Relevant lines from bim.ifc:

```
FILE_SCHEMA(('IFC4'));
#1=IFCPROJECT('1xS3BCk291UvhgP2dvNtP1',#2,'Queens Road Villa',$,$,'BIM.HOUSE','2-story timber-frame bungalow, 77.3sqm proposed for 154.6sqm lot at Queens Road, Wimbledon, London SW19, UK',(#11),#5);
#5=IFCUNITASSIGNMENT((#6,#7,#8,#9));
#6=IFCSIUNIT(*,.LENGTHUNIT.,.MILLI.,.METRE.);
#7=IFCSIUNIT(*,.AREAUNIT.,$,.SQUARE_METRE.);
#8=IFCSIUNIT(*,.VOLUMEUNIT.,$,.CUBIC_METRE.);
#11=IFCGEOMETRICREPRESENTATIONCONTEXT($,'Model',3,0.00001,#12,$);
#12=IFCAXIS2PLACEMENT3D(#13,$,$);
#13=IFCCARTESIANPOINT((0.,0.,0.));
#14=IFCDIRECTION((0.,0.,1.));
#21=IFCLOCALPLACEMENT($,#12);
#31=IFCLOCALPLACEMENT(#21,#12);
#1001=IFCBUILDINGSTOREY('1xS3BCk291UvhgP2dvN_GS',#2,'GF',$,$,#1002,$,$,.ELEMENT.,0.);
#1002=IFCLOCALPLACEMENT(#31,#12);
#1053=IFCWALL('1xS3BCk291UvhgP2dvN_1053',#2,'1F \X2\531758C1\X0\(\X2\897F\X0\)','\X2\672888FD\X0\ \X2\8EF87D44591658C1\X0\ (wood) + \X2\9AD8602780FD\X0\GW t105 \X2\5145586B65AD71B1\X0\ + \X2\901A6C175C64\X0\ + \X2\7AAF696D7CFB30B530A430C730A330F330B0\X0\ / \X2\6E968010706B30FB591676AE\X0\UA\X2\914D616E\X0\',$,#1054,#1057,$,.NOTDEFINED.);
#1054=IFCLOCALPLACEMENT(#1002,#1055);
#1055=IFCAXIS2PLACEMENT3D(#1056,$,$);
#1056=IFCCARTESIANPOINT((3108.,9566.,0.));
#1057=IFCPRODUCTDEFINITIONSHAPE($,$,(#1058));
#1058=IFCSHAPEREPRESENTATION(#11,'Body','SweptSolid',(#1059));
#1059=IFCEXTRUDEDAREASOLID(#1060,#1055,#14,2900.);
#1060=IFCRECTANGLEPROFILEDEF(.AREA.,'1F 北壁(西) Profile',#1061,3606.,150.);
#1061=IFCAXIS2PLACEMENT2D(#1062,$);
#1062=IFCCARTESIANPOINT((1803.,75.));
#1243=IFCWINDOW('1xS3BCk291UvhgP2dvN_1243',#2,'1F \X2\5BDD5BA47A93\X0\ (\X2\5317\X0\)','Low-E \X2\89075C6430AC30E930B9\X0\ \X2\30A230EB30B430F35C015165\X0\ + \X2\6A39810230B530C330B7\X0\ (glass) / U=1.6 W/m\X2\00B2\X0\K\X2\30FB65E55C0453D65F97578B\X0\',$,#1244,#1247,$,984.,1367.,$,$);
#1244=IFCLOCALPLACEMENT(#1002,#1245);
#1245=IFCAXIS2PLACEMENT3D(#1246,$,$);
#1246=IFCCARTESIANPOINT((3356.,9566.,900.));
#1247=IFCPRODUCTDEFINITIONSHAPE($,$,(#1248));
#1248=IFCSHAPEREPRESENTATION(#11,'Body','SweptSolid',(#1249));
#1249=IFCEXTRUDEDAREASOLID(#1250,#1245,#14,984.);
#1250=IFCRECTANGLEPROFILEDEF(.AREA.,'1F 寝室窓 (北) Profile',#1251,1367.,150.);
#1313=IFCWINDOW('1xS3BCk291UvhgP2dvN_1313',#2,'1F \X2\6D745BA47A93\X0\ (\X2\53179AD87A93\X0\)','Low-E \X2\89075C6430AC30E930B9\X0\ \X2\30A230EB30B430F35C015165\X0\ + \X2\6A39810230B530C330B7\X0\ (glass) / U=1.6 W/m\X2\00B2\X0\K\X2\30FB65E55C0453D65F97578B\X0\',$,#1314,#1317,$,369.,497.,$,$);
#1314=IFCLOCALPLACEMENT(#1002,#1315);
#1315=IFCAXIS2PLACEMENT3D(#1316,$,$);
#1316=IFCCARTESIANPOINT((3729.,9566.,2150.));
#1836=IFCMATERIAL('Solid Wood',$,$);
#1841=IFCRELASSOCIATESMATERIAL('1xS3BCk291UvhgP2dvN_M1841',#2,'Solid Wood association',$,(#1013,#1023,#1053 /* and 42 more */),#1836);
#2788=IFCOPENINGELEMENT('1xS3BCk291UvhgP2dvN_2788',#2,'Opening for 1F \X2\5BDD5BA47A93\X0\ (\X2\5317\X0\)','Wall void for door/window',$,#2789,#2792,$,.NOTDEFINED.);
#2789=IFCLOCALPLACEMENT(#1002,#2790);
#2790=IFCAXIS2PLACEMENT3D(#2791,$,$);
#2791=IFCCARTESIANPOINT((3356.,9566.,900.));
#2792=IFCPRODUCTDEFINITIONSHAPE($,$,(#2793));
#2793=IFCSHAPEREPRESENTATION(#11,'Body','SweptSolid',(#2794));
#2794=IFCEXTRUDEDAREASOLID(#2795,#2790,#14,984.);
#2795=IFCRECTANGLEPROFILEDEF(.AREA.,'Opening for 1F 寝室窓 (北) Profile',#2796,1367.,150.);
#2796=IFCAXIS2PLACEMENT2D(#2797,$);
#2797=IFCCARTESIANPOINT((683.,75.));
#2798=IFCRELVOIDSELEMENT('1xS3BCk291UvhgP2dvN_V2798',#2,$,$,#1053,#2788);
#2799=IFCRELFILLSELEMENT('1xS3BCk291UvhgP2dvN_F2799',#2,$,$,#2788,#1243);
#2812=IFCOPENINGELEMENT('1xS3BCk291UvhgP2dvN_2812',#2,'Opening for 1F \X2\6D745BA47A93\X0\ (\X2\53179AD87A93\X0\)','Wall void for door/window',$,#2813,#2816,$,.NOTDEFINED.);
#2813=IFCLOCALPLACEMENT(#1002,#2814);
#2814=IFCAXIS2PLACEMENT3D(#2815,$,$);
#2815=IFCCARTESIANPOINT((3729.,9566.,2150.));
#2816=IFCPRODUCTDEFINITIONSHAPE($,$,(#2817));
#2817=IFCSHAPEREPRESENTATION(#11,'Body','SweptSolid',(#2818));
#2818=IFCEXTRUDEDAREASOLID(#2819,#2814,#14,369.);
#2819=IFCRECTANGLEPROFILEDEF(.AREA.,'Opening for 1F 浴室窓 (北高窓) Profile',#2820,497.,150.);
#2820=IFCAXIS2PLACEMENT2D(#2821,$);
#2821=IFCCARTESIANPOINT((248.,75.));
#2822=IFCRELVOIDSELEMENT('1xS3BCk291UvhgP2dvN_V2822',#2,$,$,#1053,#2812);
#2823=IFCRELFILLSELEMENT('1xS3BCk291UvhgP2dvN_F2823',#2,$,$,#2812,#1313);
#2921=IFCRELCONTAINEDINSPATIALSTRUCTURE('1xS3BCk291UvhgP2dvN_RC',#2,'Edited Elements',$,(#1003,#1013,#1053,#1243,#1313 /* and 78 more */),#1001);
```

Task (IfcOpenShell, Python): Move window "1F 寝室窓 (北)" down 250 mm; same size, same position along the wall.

```python
import numpy as np
import ifcopenshell
import ifcopenshell.api.geometry
import ifcopenshell.util.placement
import ifcopenshell.util.unit

model = ifcopenshell.open("bim.ifc")
unit_scale = ifcopenshell.util.unit.calculate_unit_scale(model)

window = model.by_id(1243)
opening = window.FillsVoids[0].RelatingOpeningElement
dz = -250.0

shift = np.array([0.0, 0.0, dz])
# The window is not placed relative to its opening, so move both.
for product in (opening, window):
    matrix = ifcopenshell.util.placement.get_local_placement(product.ObjectPlacement)
    matrix[:3, 3] += shift
    ifcopenshell.api.geometry.edit_object_placement(model, product=product, matrix=matrix, is_si=False)

print(f"moved by {dz * unit_scale:+.3f} m")

model.write("bim_rev.ifc")
```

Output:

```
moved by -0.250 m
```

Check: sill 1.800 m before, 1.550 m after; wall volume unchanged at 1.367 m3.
